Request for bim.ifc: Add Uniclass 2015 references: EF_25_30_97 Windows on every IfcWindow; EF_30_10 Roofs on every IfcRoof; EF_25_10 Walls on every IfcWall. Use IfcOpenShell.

First a look at what the model holds.

```python
import ifcopenshell

model = ifcopenshell.open("bim.ifc")
print(model.schema)
print("classifications:", [c.Name for c in model.by_type("IfcClassification")])
for ifc_class in ("IfcDoor", "IfcRoof", "IfcStair", "IfcWall", "IfcWindow"):
    print(ifc_class, len(model.by_type(ifc_class)))
```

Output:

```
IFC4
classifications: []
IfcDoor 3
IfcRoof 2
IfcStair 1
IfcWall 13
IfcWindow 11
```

```python
import ifcopenshell
import ifcopenshell.api.classification

model = ifcopenshell.open("bim.ifc")

system = ifcopenshell.api.classification.add_classification(model, classification="Uniclass 2015")

codes = {
    "IfcWindow": ("EF_25_30_97", "Windows"),
    "IfcRoof": ("EF_30_10", "Roofs"),
    "IfcWall": ("EF_25_10", "Walls"),
}
for ifc_class, (code, name) in codes.items():
    products = model.by_type(ifc_class)
    ifcopenshell.api.classification.add_reference(
        model, products=products, classification=system, identification=code, name=name
    )
    print(code, len(products))

model.write("bim-out.ifc")
```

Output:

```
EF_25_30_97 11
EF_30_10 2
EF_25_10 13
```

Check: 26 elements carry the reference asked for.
